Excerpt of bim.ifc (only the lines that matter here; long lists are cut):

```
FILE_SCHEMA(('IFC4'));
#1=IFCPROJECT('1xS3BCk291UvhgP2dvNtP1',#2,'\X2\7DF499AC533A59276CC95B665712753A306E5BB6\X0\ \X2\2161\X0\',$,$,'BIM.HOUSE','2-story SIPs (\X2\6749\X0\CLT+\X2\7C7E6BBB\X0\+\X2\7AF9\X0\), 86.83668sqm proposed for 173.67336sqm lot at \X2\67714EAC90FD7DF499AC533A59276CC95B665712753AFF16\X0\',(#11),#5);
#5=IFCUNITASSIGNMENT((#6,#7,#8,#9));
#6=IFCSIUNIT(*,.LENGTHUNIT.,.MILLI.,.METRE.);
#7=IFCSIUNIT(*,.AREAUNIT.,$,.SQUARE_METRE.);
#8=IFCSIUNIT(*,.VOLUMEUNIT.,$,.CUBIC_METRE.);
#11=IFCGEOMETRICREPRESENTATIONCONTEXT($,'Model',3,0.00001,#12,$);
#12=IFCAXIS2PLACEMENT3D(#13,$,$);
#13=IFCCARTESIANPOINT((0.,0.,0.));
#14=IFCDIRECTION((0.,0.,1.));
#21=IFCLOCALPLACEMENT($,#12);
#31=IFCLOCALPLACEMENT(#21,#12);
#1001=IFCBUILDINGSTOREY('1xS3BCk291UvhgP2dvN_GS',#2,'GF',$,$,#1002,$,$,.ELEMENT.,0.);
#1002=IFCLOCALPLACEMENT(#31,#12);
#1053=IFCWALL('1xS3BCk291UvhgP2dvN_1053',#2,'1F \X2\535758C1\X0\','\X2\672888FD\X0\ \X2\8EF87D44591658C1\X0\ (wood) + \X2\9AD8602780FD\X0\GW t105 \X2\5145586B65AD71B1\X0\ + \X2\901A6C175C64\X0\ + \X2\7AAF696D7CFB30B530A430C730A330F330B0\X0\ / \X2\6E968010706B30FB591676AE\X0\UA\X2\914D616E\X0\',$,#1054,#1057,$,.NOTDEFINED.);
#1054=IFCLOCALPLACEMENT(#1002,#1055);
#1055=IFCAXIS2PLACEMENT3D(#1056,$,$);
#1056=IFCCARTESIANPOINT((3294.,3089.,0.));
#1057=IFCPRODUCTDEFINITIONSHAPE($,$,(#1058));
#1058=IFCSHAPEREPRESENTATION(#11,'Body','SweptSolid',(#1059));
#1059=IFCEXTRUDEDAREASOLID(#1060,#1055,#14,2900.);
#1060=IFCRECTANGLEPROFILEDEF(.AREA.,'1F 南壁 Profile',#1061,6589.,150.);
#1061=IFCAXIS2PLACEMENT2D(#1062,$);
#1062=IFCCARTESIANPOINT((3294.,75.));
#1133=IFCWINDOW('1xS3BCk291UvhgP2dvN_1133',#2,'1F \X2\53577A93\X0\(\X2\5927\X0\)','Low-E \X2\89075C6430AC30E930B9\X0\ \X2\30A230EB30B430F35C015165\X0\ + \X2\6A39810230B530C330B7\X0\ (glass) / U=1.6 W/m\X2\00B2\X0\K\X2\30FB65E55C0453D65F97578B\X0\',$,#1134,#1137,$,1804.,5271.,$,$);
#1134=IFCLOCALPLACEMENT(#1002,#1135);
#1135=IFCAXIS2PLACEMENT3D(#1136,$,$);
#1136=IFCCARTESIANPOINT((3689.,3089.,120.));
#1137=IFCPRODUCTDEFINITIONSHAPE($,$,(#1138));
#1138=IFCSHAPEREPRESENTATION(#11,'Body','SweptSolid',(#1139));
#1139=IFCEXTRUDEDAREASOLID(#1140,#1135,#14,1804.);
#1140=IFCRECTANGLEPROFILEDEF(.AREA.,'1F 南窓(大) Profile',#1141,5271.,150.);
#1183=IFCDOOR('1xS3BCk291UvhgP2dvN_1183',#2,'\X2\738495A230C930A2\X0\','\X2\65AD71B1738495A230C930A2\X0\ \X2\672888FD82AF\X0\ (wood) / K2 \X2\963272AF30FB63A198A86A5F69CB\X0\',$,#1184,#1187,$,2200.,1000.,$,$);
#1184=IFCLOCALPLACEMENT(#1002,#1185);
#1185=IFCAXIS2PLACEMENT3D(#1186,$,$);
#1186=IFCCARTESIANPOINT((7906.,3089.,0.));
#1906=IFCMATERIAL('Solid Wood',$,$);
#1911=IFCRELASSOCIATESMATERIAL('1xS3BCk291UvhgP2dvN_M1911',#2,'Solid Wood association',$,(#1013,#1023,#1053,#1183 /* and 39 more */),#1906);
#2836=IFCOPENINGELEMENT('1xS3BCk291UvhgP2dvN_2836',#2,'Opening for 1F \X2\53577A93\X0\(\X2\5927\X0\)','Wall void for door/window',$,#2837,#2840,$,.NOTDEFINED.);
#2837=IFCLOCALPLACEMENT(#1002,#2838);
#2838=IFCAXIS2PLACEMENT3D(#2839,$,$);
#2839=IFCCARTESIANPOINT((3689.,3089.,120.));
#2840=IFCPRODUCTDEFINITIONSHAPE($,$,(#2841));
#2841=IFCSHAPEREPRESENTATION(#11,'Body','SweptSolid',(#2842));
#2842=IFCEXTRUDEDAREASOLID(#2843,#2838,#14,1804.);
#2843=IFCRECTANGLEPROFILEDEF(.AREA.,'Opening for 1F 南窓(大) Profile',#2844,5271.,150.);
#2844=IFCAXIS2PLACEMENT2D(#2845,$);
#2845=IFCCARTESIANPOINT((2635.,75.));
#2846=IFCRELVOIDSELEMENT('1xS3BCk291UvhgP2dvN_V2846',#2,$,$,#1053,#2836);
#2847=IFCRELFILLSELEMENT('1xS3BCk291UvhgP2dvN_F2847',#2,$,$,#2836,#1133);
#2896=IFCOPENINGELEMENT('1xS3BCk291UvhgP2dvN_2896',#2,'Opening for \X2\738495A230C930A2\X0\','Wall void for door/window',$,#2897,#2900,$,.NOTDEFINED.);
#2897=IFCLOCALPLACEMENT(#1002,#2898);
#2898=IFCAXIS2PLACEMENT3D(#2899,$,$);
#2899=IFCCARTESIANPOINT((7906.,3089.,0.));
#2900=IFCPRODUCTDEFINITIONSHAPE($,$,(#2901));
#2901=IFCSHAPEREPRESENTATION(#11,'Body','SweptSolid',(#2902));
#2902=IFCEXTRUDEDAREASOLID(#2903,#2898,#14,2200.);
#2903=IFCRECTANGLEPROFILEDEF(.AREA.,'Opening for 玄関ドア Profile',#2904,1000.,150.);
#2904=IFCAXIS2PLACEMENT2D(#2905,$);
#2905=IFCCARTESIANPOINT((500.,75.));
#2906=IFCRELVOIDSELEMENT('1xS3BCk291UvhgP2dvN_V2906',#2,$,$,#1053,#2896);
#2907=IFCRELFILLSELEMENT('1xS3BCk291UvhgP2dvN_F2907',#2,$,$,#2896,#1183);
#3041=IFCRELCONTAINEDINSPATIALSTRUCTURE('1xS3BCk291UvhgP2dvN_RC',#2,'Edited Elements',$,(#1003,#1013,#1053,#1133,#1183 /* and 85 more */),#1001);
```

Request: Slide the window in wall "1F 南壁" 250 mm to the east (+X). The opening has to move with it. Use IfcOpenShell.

```python
import ifcopenshell
import ifcopenshell.api.geometry
import ifcopenshell.util.placement

model = ifcopenshell.open("bim.ifc")

window = model.by_guid("1xS3BCk291UvhgP2dvN_1133")
opening = window.FillsVoids[0].RelatingOpeningElement
wall = opening.VoidsElements[0].RelatingBuildingElement

wall_matrix = ifcopenshell.util.placement.get_local_placement(wall.ObjectPlacement)
shift = wall_matrix[:3, 0] * 250.0
before = ifcopenshell.util.placement.get_local_placement(window.ObjectPlacement)[:3, 3].copy()

# The window is not placed relative to its opening, so move both.
for product in (opening, window):
    matrix = ifcopenshell.util.placement.get_local_placement(product.ObjectPlacement)
    matrix[:3, 3] += shift
    ifcopenshell.api.geometry.edit_object_placement(model, product=product, matrix=matrix, is_si=False)

after = ifcopenshell.util.placement.get_local_placement(window.ObjectPlacement)[:3, 3]
print("window moved by", (after - before).round(3) + 0.0)

model.write("bim_edited.ifc")
```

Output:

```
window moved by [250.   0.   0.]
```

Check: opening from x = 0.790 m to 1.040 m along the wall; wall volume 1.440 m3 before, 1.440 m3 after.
